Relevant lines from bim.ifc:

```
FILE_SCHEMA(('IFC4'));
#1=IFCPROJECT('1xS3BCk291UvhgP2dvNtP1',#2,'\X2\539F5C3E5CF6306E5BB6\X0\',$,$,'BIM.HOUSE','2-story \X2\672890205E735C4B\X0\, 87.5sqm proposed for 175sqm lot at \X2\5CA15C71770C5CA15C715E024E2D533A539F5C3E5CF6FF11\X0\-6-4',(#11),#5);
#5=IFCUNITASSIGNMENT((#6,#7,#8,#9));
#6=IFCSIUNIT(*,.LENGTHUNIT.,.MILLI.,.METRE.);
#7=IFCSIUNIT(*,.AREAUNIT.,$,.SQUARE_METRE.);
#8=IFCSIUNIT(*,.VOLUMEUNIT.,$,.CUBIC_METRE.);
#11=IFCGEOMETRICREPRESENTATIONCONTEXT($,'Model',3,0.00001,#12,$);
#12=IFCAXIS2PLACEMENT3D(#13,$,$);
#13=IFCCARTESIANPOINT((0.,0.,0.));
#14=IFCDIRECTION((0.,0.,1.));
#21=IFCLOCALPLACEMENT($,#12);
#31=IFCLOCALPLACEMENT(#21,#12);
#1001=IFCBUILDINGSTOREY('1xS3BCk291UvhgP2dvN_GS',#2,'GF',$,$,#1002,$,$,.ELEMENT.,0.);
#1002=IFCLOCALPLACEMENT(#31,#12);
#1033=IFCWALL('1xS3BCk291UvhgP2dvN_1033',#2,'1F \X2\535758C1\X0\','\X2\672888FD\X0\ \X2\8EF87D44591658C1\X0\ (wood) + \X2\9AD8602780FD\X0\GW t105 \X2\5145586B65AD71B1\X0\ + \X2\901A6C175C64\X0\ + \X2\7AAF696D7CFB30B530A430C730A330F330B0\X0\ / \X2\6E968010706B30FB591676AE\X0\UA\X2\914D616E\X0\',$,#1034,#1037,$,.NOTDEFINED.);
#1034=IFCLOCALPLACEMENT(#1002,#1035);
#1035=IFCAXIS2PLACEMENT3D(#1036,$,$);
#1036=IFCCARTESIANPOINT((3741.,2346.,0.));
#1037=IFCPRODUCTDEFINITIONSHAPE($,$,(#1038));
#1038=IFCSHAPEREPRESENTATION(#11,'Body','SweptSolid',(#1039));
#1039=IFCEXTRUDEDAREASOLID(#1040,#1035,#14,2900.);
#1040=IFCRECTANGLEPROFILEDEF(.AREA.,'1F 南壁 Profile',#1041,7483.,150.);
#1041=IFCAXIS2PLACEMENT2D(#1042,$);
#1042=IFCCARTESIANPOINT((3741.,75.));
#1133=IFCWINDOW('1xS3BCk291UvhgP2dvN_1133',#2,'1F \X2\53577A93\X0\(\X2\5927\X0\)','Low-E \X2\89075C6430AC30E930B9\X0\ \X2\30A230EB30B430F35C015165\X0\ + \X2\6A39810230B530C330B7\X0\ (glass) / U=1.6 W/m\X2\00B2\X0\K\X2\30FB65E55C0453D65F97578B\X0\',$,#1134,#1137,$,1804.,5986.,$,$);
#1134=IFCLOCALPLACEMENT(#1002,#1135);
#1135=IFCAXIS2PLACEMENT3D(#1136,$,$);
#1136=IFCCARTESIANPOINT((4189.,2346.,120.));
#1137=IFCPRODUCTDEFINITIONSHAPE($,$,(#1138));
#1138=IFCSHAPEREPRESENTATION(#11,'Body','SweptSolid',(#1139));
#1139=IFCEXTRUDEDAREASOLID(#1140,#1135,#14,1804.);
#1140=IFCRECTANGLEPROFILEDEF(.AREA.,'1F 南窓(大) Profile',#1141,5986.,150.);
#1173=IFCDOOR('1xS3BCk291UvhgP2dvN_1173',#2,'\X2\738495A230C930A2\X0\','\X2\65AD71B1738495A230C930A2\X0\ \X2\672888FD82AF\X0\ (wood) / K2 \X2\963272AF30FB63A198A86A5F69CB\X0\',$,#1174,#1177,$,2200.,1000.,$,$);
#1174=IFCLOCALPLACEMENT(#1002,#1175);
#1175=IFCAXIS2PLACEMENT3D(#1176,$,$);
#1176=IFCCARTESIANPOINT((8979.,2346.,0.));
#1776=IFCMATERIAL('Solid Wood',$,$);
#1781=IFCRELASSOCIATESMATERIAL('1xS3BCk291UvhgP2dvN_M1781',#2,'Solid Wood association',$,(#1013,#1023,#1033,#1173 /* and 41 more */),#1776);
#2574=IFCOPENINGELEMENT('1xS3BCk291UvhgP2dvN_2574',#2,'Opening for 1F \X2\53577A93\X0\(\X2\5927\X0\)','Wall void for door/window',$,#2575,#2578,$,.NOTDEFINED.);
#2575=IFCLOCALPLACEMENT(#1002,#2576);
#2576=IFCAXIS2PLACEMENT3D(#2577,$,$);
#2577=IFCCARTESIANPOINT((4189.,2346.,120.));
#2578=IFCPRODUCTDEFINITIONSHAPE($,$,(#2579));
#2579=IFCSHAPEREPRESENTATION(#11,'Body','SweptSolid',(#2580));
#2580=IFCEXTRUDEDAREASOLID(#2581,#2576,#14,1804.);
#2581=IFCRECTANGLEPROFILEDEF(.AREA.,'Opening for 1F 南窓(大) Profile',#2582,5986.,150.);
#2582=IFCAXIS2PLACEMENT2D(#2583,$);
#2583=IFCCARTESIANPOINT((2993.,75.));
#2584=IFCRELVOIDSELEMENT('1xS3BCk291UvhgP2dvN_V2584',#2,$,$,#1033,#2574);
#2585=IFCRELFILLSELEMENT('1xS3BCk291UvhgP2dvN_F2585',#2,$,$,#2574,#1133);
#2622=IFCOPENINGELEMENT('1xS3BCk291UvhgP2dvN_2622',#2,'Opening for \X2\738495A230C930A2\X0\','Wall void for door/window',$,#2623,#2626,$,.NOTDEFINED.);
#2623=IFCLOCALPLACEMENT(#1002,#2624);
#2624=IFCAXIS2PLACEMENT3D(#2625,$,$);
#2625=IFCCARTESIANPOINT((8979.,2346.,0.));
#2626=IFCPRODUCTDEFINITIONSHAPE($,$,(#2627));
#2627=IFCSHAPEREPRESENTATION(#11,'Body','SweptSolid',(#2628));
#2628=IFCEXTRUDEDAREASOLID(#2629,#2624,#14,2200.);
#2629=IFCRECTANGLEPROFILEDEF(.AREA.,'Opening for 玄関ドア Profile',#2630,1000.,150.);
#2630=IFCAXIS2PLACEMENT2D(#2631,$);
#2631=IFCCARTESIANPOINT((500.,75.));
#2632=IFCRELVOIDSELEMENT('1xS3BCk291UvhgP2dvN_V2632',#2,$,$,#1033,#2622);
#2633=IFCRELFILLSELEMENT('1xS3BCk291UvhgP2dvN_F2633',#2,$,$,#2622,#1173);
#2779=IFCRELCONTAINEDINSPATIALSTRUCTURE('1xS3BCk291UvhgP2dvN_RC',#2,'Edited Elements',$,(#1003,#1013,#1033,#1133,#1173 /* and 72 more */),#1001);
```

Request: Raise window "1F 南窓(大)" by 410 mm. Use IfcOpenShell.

```python
import numpy as np
import ifcopenshell
import ifcopenshell.api.geometry
import ifcopenshell.util.placement
import ifcopenshell.util.unit

model = ifcopenshell.open("bim.ifc")
unit_scale = ifcopenshell.util.unit.calculate_unit_scale(model)

window = model.by_id(1133)
opening = window.FillsVoids[0].RelatingOpeningElement
dz = 0.41 / unit_scale

shift = np.array([0.0, 0.0, dz])
# The window is not placed relative to its opening, so move both.
for product in (opening, window):
    matrix = ifcopenshell.util.placement.get_local_placement(product.ObjectPlacement)
    matrix[:3, 3] += shift
    ifcopenshell.api.geometry.edit_object_placement(model, product=product, matrix=matrix, is_si=False)

print(f"moved by {dz * unit_scale:+.3f} m")

model.write("bim_rev.ifc")
```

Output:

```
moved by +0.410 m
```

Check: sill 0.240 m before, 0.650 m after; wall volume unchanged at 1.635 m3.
